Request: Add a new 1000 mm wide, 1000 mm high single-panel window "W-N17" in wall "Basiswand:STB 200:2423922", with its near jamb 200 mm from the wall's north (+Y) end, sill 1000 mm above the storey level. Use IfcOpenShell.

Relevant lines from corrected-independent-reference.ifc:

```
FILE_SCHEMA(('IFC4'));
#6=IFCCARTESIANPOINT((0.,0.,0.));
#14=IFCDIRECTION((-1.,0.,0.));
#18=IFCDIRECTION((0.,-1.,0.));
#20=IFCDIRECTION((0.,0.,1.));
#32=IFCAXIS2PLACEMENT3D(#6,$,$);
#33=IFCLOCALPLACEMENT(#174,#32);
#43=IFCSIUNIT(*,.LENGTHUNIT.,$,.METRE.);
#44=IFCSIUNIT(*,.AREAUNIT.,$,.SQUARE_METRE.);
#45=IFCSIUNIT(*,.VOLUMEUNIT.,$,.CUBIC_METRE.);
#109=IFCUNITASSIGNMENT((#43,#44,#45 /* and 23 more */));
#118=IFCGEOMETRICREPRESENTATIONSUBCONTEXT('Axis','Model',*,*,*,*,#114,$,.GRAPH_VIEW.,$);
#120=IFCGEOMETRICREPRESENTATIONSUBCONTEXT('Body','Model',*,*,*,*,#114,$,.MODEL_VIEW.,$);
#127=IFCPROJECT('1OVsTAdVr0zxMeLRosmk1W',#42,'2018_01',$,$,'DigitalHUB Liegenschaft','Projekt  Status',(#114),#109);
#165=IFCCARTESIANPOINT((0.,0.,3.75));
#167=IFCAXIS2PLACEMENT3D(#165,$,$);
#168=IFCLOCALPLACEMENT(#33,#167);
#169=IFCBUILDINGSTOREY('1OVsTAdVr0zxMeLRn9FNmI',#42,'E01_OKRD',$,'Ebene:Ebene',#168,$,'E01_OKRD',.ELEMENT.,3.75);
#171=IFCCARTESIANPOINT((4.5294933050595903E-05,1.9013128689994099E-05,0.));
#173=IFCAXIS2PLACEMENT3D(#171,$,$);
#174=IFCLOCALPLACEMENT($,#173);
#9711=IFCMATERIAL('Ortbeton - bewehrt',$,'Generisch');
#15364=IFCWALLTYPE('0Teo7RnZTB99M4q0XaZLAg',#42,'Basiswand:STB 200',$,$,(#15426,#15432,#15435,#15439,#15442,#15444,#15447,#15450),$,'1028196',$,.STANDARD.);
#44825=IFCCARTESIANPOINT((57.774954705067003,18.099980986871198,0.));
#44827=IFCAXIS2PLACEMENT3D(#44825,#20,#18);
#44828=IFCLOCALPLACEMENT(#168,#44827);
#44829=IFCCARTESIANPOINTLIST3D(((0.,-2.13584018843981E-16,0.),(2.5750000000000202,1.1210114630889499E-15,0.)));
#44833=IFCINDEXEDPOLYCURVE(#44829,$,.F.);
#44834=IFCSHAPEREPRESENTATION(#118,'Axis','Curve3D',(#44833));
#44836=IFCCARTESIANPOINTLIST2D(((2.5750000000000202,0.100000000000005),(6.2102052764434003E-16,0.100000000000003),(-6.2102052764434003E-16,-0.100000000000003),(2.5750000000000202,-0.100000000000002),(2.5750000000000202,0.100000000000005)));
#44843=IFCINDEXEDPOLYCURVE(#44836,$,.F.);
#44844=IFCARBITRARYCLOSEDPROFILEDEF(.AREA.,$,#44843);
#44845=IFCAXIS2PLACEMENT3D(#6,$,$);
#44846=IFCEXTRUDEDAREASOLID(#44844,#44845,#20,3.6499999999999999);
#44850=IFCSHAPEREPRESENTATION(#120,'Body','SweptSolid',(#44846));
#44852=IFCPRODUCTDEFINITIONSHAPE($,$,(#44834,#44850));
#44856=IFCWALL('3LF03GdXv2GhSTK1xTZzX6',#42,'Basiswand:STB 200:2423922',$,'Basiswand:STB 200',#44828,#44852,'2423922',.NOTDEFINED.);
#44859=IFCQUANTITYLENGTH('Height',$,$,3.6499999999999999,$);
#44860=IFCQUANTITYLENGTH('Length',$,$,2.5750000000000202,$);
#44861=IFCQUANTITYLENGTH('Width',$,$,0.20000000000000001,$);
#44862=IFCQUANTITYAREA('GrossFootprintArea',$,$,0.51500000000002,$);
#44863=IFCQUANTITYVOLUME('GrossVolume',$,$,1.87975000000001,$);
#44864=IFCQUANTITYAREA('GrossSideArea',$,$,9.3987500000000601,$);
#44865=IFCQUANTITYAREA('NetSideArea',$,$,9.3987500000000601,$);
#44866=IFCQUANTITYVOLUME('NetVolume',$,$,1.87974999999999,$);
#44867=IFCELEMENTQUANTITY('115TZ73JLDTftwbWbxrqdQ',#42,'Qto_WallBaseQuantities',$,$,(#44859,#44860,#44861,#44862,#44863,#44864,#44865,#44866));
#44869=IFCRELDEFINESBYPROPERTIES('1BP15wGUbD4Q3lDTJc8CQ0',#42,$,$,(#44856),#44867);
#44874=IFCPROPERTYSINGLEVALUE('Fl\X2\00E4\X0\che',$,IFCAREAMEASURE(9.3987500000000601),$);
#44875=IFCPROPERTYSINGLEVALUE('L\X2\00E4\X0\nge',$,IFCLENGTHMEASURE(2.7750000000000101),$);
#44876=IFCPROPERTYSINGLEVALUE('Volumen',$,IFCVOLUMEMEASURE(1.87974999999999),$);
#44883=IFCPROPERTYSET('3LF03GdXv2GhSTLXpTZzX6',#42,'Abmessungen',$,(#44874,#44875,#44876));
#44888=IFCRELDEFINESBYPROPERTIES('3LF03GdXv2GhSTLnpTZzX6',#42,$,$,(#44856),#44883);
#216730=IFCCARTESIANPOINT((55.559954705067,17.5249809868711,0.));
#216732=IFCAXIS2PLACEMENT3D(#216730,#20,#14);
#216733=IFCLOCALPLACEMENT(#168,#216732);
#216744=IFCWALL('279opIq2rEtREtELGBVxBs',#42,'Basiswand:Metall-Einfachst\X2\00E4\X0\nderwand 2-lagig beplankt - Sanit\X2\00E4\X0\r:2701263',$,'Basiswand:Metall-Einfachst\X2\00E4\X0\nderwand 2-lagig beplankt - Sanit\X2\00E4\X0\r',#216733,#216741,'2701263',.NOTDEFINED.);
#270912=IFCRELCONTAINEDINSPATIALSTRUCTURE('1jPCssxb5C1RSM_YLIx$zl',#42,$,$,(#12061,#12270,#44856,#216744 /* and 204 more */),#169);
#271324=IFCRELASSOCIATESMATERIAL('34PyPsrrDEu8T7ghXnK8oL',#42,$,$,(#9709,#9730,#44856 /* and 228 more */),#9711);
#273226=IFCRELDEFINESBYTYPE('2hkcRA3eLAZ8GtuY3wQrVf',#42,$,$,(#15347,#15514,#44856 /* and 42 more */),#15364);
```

```python
import numpy as np
import ifcopenshell
import ifcopenshell.api.feature
import ifcopenshell.api.geometry
import ifcopenshell.api.pset
import ifcopenshell.api.root
import ifcopenshell.api.spatial
import ifcopenshell.geom
import ifcopenshell.util.element
import ifcopenshell.util.placement
import ifcopenshell.util.representation
import ifcopenshell.util.shape
import ifcopenshell.util.unit

model = ifcopenshell.open("corrected-independent-reference.ifc")
unit_scale = ifcopenshell.util.unit.calculate_unit_scale(model)
area_scale = ifcopenshell.util.unit.calculate_unit_scale(model, "AREAUNIT")
volume_scale = ifcopenshell.util.unit.calculate_unit_scale(model, "VOLUMEUNIT")
settings = ifcopenshell.geom.settings()


def volume(element):
    """Net volume in cubic metres, openings subtracted."""
    shape = ifcopenshell.geom.create_shape(settings, element)
    return ifcopenshell.util.shape.get_volume(shape.geometry)


wall = model.by_id(44856)
storey = ifcopenshell.util.element.get_container(wall, ifc_class="IfcBuildingStorey")
context = ifcopenshell.util.representation.get_context(model, "Model", "Body", "MODEL_VIEW")
before = volume(wall)

width, height, from_end, sill = 1, 1, 0.2, 1  # metres

# The wall runs along its own X axis, and the end named is its -X end.
wall_shape = ifcopenshell.geom.create_shape(settings, wall)
x, y, z = ifcopenshell.util.shape.get_vertices(wall_shape.geometry).T
start = x.min() + from_end
face, thickness = float(y.min()), float(y.max() - y.min())
wall_matrix = ifcopenshell.util.placement.get_local_placement(wall.ObjectPlacement)
level = ifcopenshell.util.placement.get_local_placement(storey.ObjectPlacement)[2, 3]


def in_wall(x, y):
    """Placement at x, y metres in the wall's axes, at sill height."""
    matrix = wall_matrix.copy()
    matrix[:, 3] = wall_matrix @ np.array([x / unit_scale, y / unit_scale, 0.0, 1.0])
    matrix[2, 3] = level + sill / unit_scale
    return matrix


# Opening: a box that overshoots both wall faces by 50 mm.
opening = ifcopenshell.api.root.create_entity(model, ifc_class="IfcOpeningElement", predefined_type="OPENING")
box = ifcopenshell.api.geometry.add_wall_representation(
    model, context=context, length=width, height=height, thickness=thickness + 0.1
)
ifcopenshell.api.geometry.assign_representation(model, product=opening, representation=box)
ifcopenshell.api.geometry.edit_object_placement(model, product=opening, matrix=in_wall(start, face - 0.05), is_si=False)
ifcopenshell.api.feature.add_feature(model, feature=opening, element=wall)

window = ifcopenshell.api.root.create_entity(model, ifc_class="IfcWindow", name="W-N17", predefined_type="WINDOW")
window.OverallWidth, window.OverallHeight = width / unit_scale, height / unit_scale
window.PartitioningType = "SINGLE_PANEL"
body = ifcopenshell.api.geometry.add_window_representation(
    model,
    context=context,
    overall_width=window.OverallWidth,
    overall_height=window.OverallHeight,
    partition_type="SINGLE_PANEL",
)
ifcopenshell.api.geometry.assign_representation(model, product=window, representation=body)
ifcopenshell.api.spatial.assign_container(model, products=[window], relating_structure=storey)
ifcopenshell.api.feature.add_filling(model, opening=opening, element=window)

# Centre the window in the wall's thickness.
ifcopenshell.api.geometry.edit_object_placement(model, product=window, matrix=in_wall(start, face), is_si=False)
window_shape = ifcopenshell.geom.create_shape(settings, window)
depth = ifcopenshell.util.shape.get_vertices(window_shape.geometry)[:, 1]
offset = face + thickness / 2 - (depth.min() + depth.max()) / 2
ifcopenshell.api.geometry.edit_object_placement(model, product=window, matrix=in_wall(start, offset), is_si=False)

after = volume(wall)

# Update the wall's stored quantities.
qto = model.by_id(ifcopenshell.util.element.get_pset(wall, "Qto_WallBaseQuantities", should_inherit=False)["id"])
ifcopenshell.api.pset.edit_qto(model, qto=qto, properties={
    "NetSideArea": after / thickness / area_scale,
    "NetVolume": after / volume_scale,
})
pset = model.by_id(ifcopenshell.util.element.get_pset(wall, "Abmessungen", should_inherit=False)["id"])
ifcopenshell.api.pset.edit_pset(model, pset=pset, properties={
    "Fläche": model.create_entity("IfcAreaMeasure", after / thickness / area_scale),
    "Volumen": model.create_entity("IfcVolumeMeasure", after / volume_scale),
})

print(f"wall volume {before:.3f} -> {after:.3f} m3")

model.write("corrected-independent-reference_edited.ifc")
```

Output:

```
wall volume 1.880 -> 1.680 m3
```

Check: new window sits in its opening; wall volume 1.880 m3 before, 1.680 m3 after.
